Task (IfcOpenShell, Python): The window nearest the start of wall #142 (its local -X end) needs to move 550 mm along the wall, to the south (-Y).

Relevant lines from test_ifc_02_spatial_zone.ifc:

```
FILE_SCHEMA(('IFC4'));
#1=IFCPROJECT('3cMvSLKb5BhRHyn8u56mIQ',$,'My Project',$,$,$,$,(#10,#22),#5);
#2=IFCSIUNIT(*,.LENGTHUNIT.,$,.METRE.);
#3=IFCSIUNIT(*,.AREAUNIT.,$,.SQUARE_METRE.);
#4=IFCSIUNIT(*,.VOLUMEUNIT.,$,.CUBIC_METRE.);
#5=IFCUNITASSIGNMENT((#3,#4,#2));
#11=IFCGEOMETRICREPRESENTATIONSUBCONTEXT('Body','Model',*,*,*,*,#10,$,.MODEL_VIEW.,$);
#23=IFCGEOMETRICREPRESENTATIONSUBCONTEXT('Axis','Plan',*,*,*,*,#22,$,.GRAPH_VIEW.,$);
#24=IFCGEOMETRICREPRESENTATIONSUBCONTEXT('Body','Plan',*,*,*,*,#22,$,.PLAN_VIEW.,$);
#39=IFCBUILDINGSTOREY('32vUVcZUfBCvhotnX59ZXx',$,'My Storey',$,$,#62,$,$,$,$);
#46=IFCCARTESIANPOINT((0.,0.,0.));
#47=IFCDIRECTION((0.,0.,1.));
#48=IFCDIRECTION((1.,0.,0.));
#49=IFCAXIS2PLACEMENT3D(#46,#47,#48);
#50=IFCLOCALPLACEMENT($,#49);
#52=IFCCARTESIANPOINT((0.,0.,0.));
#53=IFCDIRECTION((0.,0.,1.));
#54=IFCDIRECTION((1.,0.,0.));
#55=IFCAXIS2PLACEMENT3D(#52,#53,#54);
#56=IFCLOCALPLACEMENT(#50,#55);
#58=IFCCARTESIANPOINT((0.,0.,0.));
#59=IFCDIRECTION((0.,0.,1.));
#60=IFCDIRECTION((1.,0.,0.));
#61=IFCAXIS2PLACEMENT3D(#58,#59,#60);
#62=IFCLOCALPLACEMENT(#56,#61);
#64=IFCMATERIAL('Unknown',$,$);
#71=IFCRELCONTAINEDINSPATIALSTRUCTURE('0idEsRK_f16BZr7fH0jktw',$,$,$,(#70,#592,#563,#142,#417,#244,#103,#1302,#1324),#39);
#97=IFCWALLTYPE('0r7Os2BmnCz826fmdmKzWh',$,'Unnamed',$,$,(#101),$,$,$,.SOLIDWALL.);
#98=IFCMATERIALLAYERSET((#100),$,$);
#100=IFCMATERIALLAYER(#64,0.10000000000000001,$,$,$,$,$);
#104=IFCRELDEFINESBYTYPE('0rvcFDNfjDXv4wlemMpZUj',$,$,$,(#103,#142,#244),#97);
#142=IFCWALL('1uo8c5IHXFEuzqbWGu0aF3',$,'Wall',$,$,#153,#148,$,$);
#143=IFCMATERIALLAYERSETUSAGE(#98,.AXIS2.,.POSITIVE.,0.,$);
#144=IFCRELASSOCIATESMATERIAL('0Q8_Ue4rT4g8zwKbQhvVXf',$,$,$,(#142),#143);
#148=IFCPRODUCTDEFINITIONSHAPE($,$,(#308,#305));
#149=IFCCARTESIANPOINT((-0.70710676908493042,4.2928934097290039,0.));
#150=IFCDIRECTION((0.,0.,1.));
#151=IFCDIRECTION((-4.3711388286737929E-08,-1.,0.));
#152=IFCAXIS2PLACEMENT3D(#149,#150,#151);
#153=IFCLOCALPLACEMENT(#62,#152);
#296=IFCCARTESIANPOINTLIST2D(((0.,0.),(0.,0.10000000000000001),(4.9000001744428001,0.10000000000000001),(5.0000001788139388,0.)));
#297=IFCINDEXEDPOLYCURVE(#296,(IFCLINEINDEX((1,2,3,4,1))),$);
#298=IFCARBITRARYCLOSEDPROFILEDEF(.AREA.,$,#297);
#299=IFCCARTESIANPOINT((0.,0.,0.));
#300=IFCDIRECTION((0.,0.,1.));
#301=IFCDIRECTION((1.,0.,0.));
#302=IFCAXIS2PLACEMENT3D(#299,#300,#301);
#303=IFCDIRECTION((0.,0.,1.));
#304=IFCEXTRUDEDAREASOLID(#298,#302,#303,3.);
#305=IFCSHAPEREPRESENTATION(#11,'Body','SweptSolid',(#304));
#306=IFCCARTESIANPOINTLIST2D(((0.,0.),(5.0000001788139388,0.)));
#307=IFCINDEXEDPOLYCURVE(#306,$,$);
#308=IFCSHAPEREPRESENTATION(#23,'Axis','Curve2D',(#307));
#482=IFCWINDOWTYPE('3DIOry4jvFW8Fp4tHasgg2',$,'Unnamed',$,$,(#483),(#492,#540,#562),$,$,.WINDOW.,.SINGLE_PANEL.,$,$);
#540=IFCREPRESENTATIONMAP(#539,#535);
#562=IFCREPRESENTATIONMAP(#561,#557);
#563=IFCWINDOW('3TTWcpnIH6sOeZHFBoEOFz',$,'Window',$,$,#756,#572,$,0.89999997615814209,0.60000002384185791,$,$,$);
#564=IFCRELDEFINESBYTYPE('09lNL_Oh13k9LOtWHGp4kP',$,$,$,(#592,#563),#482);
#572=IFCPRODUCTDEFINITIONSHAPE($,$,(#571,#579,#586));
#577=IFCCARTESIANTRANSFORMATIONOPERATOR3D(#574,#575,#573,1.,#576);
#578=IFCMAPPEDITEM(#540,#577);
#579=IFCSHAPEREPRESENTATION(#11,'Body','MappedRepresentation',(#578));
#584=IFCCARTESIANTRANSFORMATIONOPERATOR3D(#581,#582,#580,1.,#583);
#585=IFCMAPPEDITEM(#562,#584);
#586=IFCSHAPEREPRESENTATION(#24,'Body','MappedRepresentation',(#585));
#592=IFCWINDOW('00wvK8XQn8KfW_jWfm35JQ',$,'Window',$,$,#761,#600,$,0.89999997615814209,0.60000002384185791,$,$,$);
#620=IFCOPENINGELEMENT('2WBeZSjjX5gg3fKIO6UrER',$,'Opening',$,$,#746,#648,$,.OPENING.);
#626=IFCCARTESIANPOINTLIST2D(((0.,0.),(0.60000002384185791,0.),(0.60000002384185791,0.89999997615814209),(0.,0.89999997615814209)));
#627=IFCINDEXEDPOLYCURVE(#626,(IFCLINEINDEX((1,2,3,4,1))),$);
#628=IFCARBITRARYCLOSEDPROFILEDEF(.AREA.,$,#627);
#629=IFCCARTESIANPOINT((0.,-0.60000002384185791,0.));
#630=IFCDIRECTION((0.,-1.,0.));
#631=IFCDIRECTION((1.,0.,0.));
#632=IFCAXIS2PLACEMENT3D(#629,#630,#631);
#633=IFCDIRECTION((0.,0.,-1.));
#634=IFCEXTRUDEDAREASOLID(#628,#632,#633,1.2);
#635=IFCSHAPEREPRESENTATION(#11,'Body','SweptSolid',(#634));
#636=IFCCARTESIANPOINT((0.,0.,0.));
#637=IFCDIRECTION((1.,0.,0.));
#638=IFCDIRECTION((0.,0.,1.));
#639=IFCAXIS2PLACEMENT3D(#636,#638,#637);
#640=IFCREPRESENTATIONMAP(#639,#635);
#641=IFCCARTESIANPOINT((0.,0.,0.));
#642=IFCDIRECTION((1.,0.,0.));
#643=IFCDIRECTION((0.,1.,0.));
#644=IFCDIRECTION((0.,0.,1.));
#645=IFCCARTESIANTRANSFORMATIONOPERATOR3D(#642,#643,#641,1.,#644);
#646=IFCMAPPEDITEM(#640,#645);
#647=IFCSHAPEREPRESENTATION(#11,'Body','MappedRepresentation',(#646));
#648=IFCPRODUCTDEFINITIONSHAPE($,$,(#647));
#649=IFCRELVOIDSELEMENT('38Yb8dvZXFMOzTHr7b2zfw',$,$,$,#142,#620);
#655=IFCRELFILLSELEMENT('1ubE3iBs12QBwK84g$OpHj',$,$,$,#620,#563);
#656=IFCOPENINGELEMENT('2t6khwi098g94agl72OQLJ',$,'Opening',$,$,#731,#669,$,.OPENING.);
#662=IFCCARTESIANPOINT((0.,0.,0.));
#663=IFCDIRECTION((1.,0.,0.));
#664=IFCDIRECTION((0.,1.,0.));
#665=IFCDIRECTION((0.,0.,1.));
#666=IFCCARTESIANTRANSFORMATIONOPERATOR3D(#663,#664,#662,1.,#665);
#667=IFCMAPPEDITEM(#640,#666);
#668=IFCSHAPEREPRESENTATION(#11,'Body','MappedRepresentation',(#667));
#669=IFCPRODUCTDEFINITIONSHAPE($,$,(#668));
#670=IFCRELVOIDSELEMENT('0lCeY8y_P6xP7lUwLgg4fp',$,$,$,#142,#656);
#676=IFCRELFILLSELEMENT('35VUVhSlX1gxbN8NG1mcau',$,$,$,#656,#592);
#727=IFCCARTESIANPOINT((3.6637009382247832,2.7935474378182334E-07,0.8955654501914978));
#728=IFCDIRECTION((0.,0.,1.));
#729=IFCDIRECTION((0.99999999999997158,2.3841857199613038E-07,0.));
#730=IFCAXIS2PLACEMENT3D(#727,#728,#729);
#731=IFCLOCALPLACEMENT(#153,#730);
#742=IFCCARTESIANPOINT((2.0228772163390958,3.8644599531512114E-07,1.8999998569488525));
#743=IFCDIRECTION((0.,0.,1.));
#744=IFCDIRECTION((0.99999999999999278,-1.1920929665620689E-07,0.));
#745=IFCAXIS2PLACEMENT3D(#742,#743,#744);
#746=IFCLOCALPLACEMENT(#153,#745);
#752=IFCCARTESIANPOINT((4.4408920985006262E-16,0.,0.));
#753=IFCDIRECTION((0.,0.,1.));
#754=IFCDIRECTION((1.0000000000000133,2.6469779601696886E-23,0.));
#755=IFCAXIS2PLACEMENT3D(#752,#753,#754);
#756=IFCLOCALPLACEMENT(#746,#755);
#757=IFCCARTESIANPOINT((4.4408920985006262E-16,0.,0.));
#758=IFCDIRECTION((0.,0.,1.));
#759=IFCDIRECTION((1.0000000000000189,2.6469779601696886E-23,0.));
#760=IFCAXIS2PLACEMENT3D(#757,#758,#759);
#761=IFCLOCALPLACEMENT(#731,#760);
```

```python
import ifcopenshell
import ifcopenshell.api.geometry
import ifcopenshell.util.placement
import ifcopenshell.util.unit

model = ifcopenshell.open("test_ifc_02_spatial_zone.ifc")
unit_scale = ifcopenshell.util.unit.calculate_unit_scale(model)

window = model.by_id(563)
opening = window.FillsVoids[0].RelatingOpeningElement
wall = opening.VoidsElements[0].RelatingBuildingElement

wall_matrix = ifcopenshell.util.placement.get_local_placement(wall.ObjectPlacement)
shift = wall_matrix[:3, 0] * 0.55 / unit_scale
before = ifcopenshell.util.placement.get_local_placement(window.ObjectPlacement)[:3, 3].copy()

# The window is placed relative to its opening, so it follows when the opening moves.
matrix = ifcopenshell.util.placement.get_local_placement(opening.ObjectPlacement)
matrix[:3, 3] += shift
ifcopenshell.api.geometry.edit_object_placement(
    model, product=opening, matrix=matrix, is_si=False, should_transform_children=True
)

after = ifcopenshell.util.placement.get_local_placement(window.ObjectPlacement)[:3, 3]
print("window moved by", (after - before).round(3) + 0.0)

model.write("test_ifc_02_spatial_zone-out.ifc")
```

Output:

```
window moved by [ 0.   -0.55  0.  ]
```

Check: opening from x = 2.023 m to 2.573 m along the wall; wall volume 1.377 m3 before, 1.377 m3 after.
